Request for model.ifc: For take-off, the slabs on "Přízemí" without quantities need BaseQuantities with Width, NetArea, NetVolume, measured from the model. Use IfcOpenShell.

First a look at what the model holds.

```python
import ifcopenshell
import ifcopenshell.util.element
import ifcopenshell.util.unit

model = ifcopenshell.open("model.ifc")
print(model.schema)
for unit_type in ("LENGTHUNIT", "AREAUNIT", "VOLUMEUNIT"):
    print(unit_type, ifcopenshell.util.unit.calculate_unit_scale(model, unit_type))
storey = next(s for s in model.by_type("IfcBuildingStorey") if s.Name == "Přízemí")
slabs = [e for e in ifcopenshell.util.element.get_decomposition(storey) if e.is_a("IfcSlab")]
for e in sorted(slabs, key=lambda e: e.id()):
    print(e.id(), e.is_a(), e.Name, list(ifcopenshell.util.element.get_psets(e, qtos_only=True)), sep=" | ")
```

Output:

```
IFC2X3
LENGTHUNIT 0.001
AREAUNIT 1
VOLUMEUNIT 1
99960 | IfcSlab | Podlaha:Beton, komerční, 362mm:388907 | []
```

```python
import ifcopenshell
import ifcopenshell.api.pset
import ifcopenshell.geom
import ifcopenshell.util.element
import ifcopenshell.util.shape
import ifcopenshell.util.unit

model = ifcopenshell.open("model.ifc")
unit_scale = ifcopenshell.util.unit.calculate_unit_scale(model)
area_scale = ifcopenshell.util.unit.calculate_unit_scale(model, "AREAUNIT")
volume_scale = ifcopenshell.util.unit.calculate_unit_scale(model, "VOLUMEUNIT")
settings = ifcopenshell.geom.settings()

storey = next(s for s in model.by_type("IfcBuildingStorey") if s.Name == "Přízemí")
slabs = [e for e in ifcopenshell.util.element.get_decomposition(storey) if e.is_a("IfcSlab")]

for e in sorted(slabs, key=lambda e: e.id()):
    if ifcopenshell.util.element.get_psets(e, qtos_only=True, should_inherit=False):
        continue
    # Geometry comes back in metres, in the element's own axes.
    shape = ifcopenshell.geom.create_shape(settings, e)
    values = {
        "Width": ifcopenshell.util.shape.get_z(shape.geometry) / unit_scale,
        "NetArea": ifcopenshell.util.shape.get_footprint_area(shape.geometry) / area_scale,
        "NetVolume": ifcopenshell.util.shape.get_volume(shape.geometry) / volume_scale,
    }
    qto = ifcopenshell.api.pset.add_qto(model, product=e, name="BaseQuantities")
    ifcopenshell.api.pset.edit_qto(model, qto=qto, properties=values)
    print(e.id(), {k: round(v, 3) for k, v in values.items()})

model.write("model_edited.ifc")
```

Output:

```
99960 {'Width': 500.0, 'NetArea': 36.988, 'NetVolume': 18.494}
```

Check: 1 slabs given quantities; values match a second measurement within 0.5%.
